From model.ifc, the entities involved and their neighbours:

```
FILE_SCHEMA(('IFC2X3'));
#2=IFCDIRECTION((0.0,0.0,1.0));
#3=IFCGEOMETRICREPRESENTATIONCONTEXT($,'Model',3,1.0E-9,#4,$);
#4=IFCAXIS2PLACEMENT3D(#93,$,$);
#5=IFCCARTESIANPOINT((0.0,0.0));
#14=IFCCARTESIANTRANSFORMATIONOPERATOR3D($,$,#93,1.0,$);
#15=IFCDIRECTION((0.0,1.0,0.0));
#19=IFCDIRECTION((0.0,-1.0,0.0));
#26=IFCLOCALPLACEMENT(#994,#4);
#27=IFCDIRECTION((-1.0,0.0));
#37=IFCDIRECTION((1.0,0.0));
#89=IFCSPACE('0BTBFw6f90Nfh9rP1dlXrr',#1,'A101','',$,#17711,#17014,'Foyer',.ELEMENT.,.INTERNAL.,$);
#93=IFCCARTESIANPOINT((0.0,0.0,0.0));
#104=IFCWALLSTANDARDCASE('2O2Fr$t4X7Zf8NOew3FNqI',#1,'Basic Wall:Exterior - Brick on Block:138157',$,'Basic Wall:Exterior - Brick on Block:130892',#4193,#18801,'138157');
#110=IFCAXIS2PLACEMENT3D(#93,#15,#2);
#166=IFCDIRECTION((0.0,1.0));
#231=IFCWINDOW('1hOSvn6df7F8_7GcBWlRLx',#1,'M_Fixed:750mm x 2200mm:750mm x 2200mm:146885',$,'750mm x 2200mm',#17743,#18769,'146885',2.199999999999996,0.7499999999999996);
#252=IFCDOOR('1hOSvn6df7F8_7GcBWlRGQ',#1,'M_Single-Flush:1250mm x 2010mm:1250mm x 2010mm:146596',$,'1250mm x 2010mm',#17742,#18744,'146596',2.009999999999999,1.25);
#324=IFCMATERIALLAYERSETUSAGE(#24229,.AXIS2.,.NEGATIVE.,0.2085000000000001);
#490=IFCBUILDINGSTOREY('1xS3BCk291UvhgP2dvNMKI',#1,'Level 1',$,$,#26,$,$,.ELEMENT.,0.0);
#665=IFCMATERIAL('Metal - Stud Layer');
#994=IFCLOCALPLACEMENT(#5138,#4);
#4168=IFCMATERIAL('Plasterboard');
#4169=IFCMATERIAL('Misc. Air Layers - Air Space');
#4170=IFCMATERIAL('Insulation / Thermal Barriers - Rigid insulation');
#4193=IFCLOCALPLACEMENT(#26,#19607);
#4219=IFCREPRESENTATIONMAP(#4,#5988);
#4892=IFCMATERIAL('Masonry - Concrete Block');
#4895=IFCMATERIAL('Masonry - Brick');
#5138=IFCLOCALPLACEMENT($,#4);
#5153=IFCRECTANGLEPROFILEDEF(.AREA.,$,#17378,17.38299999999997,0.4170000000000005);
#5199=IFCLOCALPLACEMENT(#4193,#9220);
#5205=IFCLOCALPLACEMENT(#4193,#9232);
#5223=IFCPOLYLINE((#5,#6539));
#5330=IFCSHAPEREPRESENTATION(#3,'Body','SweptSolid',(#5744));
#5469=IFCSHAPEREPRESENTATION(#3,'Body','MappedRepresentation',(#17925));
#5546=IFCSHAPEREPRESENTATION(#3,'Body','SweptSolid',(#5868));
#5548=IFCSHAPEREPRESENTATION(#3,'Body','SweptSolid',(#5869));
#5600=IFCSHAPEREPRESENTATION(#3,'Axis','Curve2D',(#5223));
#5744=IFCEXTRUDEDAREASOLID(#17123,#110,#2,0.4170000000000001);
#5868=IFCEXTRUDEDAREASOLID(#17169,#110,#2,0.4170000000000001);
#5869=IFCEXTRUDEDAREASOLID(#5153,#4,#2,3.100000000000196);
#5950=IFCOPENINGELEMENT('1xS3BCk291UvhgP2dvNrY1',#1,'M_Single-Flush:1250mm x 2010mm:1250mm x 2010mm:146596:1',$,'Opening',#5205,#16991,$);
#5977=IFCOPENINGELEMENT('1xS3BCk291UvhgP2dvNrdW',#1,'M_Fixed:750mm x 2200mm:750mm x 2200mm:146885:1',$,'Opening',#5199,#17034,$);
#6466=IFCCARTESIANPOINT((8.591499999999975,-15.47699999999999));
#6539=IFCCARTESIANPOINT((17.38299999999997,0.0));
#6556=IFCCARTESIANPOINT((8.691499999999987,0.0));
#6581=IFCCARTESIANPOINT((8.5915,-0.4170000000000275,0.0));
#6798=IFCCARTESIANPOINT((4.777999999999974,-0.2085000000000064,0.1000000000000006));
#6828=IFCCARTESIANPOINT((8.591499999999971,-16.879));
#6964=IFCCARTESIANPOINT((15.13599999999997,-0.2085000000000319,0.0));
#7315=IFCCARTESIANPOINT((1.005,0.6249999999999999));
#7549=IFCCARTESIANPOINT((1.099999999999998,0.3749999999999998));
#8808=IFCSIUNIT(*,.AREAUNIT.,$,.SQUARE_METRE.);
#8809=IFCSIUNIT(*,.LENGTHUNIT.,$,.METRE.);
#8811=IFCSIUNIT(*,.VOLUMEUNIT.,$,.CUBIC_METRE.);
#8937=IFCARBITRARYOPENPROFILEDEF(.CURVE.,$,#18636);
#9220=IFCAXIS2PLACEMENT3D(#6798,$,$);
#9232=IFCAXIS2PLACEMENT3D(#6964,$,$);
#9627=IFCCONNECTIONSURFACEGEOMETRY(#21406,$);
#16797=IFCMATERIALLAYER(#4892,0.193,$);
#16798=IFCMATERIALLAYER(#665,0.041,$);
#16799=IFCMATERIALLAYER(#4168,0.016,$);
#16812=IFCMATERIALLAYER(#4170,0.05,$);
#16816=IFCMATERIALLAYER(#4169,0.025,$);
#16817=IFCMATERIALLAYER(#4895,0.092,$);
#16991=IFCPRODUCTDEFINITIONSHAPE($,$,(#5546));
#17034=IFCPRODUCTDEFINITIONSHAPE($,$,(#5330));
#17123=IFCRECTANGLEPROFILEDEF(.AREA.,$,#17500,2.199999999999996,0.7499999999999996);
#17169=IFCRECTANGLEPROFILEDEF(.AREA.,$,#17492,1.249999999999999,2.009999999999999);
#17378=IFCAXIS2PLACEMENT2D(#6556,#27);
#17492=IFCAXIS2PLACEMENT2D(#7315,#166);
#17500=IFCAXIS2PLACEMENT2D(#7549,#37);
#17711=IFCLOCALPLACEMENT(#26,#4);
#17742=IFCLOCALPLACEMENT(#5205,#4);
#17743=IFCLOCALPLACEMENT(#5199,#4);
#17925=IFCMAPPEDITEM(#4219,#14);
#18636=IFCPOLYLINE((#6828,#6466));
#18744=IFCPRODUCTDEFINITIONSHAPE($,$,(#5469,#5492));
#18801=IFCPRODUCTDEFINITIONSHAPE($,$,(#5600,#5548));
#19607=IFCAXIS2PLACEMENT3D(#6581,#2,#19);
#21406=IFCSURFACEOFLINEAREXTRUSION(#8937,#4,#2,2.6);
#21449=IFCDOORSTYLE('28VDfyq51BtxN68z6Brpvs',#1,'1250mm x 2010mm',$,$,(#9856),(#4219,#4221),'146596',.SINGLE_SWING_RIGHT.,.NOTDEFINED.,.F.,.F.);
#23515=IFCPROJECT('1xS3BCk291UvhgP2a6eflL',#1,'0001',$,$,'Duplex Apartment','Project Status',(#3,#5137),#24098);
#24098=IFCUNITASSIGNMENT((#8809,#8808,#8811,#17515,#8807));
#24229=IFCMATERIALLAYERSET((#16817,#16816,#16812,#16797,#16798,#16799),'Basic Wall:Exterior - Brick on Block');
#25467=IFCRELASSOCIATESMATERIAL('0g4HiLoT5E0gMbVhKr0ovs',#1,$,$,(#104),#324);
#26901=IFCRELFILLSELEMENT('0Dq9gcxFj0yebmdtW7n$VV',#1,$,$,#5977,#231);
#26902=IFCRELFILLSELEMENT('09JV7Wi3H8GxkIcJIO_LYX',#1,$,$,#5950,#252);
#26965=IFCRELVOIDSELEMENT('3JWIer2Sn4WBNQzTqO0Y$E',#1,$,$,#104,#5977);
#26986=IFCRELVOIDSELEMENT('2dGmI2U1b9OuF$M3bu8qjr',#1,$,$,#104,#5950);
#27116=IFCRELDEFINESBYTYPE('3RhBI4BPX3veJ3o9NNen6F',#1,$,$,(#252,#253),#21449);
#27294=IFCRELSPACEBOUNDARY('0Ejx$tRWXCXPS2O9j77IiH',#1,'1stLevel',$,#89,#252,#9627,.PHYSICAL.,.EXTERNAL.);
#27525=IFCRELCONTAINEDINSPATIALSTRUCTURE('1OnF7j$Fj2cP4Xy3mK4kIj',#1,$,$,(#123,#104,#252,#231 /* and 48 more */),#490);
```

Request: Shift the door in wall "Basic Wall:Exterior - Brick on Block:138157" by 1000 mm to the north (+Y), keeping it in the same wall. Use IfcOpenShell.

```python
import numpy as np
import ifcopenshell
import ifcopenshell.api.geometry
import ifcopenshell.util.placement
import ifcopenshell.util.unit

model = ifcopenshell.open("model.ifc")
unit_scale = ifcopenshell.util.unit.calculate_unit_scale(model)

door = model.by_id(252)
opening = door.FillsVoids[0].RelatingOpeningElement
wall = opening.VoidsElements[0].RelatingBuildingElement

wall_matrix = ifcopenshell.util.placement.get_local_placement(wall.ObjectPlacement)
shift = wall_matrix[:3, 0] * -1 / unit_scale
before = ifcopenshell.util.placement.get_local_placement(door.ObjectPlacement)[:3, 3].copy()

# The door is placed relative to its opening, so it follows when the opening moves.
matrix = ifcopenshell.util.placement.get_local_placement(opening.ObjectPlacement)
matrix[:3, 3] += shift
ifcopenshell.api.geometry.edit_object_placement(
    model, product=opening, matrix=matrix, is_si=False, should_transform_children=True
)

# Space boundary surfaces are stored in each space's coordinates; move them too.
for rel in door.ProvidesBoundaries:
    if not rel.ConnectionGeometry:
        continue
    surface = rel.ConnectionGeometry.SurfaceOnRelatingElement
    space_matrix = ifcopenshell.util.placement.get_local_placement(rel.RelatingSpace.ObjectPlacement)
    point = np.array(surface.Position.Location.Coordinates) + space_matrix[:3, :3].T @ shift
    surface.Position = model.createIfcAxis2Placement3D(
        model.createIfcCartesianPoint(point.tolist()), surface.Position.Axis, surface.Position.RefDirection
    )

after = ifcopenshell.util.placement.get_local_placement(door.ObjectPlacement)[:3, 3]
print("door moved by", (after - before).round(3) + 0.0)

model.write("model_edited.ifc")
```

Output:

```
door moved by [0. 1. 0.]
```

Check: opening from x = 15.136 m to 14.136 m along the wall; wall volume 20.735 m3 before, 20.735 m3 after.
